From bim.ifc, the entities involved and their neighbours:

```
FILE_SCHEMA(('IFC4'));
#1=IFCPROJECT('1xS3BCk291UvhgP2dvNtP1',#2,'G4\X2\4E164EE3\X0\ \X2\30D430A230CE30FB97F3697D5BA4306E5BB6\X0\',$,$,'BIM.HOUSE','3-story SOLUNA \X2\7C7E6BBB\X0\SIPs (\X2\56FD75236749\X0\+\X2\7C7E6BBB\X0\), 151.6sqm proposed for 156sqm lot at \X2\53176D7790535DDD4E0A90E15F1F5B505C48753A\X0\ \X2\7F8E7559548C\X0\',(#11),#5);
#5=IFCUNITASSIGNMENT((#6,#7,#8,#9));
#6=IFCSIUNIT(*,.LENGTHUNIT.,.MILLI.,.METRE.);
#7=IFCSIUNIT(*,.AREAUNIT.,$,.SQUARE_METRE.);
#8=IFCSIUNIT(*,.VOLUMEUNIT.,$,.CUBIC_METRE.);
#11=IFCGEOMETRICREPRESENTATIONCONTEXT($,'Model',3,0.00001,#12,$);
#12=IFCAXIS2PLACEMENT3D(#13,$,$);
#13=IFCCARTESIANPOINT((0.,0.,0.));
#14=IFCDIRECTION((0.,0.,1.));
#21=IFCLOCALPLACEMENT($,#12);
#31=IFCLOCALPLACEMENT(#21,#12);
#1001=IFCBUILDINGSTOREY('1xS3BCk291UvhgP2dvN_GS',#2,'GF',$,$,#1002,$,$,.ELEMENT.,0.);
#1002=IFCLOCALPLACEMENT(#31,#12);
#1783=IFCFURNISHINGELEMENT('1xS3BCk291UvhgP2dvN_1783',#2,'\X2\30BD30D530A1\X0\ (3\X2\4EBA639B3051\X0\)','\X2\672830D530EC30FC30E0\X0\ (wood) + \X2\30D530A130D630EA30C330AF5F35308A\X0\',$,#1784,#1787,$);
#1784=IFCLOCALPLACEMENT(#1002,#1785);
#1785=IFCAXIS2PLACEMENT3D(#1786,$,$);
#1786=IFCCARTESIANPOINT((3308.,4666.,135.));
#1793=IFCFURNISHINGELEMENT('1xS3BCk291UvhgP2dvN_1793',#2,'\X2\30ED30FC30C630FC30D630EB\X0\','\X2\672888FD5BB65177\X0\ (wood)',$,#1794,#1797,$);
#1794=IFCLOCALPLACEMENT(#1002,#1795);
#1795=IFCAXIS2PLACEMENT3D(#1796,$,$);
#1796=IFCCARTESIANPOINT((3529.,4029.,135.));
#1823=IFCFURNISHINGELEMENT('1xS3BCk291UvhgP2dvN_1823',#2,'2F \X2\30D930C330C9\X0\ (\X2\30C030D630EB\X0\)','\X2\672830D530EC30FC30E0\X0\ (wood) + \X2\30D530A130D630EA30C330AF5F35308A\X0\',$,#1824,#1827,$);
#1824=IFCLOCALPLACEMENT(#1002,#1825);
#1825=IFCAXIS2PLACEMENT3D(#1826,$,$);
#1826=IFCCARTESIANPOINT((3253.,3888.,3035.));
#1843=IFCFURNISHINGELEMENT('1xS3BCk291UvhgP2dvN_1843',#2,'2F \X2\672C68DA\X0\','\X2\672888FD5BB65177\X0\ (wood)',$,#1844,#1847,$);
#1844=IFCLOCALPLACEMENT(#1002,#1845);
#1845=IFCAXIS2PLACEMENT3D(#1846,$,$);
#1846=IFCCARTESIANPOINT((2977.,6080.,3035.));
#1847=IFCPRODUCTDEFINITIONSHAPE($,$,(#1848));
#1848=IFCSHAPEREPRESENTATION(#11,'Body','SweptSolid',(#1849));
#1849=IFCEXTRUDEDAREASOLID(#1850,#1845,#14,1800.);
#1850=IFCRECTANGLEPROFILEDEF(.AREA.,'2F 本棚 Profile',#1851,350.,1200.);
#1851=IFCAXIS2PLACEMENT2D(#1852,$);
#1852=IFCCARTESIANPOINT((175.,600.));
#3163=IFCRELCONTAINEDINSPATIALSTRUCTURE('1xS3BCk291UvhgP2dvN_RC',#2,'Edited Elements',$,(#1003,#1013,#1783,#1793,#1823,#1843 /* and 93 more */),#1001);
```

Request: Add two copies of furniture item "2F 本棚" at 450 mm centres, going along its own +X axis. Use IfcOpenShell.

```python
import ifcopenshell
import ifcopenshell.api.geometry
import ifcopenshell.api.root
import ifcopenshell.util.element
import ifcopenshell.util.placement

model = ifcopenshell.open("bim.ifc")


def reuse_history(source, copy):
    """copy_class also copies each property set's owner history, people and application; keep the originals."""
    for rel in copy.IsDefinedBy:
        if rel.is_a("IfcRelDefinesByProperties") and (history := rel.RelatingPropertyDefinition.OwnerHistory):
            rel.RelatingPropertyDefinition.OwnerHistory = source.OwnerHistory
            ifcopenshell.util.element.remove_deep2(model, history)


source = model.by_guid("1xS3BCk291UvhgP2dvN_1843")
base = ifcopenshell.util.placement.get_local_placement(source.ObjectPlacement)
step = base[:3, 0] * 450.0

for i in range(1, 3):
    copy = ifcopenshell.api.root.copy_class(model, product=source)
    copy.Representation = ifcopenshell.util.element.copy_deep(
        model, source.Representation, exclude=["IfcGeometricRepresentationContext", "IfcRepresentationMap"]
    )
    reuse_history(source, copy)
    matrix = base.copy()
    matrix[:3, 3] += i * step
    print("added at", matrix[:3, 3].round(3) + 0.0)
    ifcopenshell.api.geometry.edit_object_placement(model, product=copy, matrix=matrix, is_si=False)

model.write("bim_edited.ifc")
```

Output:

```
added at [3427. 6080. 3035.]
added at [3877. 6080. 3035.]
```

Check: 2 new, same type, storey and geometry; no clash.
